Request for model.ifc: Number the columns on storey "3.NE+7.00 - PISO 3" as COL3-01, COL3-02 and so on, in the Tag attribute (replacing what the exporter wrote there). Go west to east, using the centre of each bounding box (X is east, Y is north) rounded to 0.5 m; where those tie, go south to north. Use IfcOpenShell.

First a look at what the model holds.

```python
import ifcopenshell
import ifcopenshell.util.element
import ifcopenshell.util.placement

model = ifcopenshell.open("model.ifc")
print(model.schema)
storey = next(s for s in model.by_type("IfcBuildingStorey") if s.Name == "3.NE+7.00 - PISO 3")
columns = [e for e in ifcopenshell.util.element.get_decomposition(storey) if e.is_a("IfcColumn")]
for e in sorted(columns, key=lambda e: e.id()):
    origin = ifcopenshell.util.placement.get_local_placement(e.ObjectPlacement)[:3, 3]
    print(e.id(), e.Tag, e.Name, origin.round(2) + 0.0, sep=" | ")
```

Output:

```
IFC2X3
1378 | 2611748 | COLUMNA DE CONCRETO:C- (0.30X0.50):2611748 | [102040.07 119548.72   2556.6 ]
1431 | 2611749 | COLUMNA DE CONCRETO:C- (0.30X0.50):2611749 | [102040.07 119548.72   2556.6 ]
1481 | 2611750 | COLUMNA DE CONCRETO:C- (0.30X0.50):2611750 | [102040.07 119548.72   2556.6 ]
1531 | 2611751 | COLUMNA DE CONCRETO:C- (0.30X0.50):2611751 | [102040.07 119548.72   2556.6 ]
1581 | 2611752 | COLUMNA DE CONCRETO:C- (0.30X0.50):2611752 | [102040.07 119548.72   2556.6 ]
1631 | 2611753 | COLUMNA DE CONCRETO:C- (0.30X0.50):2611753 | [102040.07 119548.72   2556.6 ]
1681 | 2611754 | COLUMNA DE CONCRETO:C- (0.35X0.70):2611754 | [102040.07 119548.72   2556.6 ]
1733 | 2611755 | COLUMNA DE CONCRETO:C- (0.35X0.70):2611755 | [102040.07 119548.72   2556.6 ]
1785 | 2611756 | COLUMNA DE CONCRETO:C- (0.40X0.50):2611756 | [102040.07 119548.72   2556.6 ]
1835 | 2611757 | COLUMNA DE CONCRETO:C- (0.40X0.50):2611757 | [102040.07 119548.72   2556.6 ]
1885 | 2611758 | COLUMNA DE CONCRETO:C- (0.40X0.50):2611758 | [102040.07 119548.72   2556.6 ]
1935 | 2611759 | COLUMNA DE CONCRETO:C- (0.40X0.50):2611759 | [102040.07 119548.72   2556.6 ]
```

```python
import ifcopenshell
import ifcopenshell.geom
import ifcopenshell.util.element
import ifcopenshell.util.shape

model = ifcopenshell.open("model.ifc")
settings = ifcopenshell.geom.settings()
settings.set("use-world-coords", True)


def centre(element):
    shape = ifcopenshell.geom.create_shape(settings, element)
    return ifcopenshell.util.shape.get_bbox_centroid(shape.geometry)


storey = next(s for s in model.by_type("IfcBuildingStorey") if s.Name == "3.NE+7.00 - PISO 3")
columns = [e for e in ifcopenshell.util.element.get_decomposition(storey) if e.is_a("IfcColumn")]

# Insertion points can sit at a corner or the storey origin, so sort by the geometry (in metres).
centres = {e: centre(e) for e in columns}
columns.sort(key=lambda e: (round(centres[e][0] / 0.5), centres[e][1]))

for i, e in enumerate(columns, start=1):
    number = f"COL3-{i:02d}"
    e.Tag = number
    print(e.id(), number)

model.write("model-out.ifc")
```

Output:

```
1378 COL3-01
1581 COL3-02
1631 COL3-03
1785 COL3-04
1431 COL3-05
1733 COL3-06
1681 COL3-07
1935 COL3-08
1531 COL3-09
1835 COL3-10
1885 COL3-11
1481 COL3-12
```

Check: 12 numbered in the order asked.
